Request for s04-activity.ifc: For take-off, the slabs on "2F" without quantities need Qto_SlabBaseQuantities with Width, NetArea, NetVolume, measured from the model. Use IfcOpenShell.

First a look at what the model holds.

```python
import ifcopenshell
import ifcopenshell.util.element
import ifcopenshell.util.unit

model = ifcopenshell.open("s04-activity.ifc")
print(model.schema)
for unit_type in ("LENGTHUNIT", "AREAUNIT", "VOLUMEUNIT"):
    print(unit_type, ifcopenshell.util.unit.calculate_unit_scale(model, unit_type))
storey = next(s for s in model.by_type("IfcBuildingStorey") if s.Name == "2F")
slabs = [e for e in ifcopenshell.util.element.get_decomposition(storey) if e.is_a("IfcSlab")]
for e in sorted(slabs, key=lambda e: e.id()):
    print(e.id(), e.is_a(), e.Name, list(ifcopenshell.util.element.get_psets(e, qtos_only=True)), sep=" | ")
```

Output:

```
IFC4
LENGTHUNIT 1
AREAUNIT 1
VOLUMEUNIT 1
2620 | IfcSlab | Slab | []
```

```python
import ifcopenshell
import ifcopenshell.api.pset
import ifcopenshell.geom
import ifcopenshell.util.element
import ifcopenshell.util.shape
import ifcopenshell.util.unit

model = ifcopenshell.open("s04-activity.ifc")
unit_scale = ifcopenshell.util.unit.calculate_unit_scale(model)
area_scale = ifcopenshell.util.unit.calculate_unit_scale(model, "AREAUNIT")
volume_scale = ifcopenshell.util.unit.calculate_unit_scale(model, "VOLUMEUNIT")
settings = ifcopenshell.geom.settings()

storey = next(s for s in model.by_type("IfcBuildingStorey") if s.Name == "2F")
slabs = [e for e in ifcopenshell.util.element.get_decomposition(storey) if e.is_a("IfcSlab")]

for e in sorted(slabs, key=lambda e: e.id()):
    if ifcopenshell.util.element.get_psets(e, qtos_only=True, should_inherit=False):
        continue
    # Geometry comes back in metres, in the element's own axes.
    shape = ifcopenshell.geom.create_shape(settings, e)
    values = {
        "Width": ifcopenshell.util.shape.get_z(shape.geometry) / unit_scale,
        "NetArea": ifcopenshell.util.shape.get_footprint_area(shape.geometry) / area_scale,
        "NetVolume": ifcopenshell.util.shape.get_volume(shape.geometry) / volume_scale,
    }
    qto = ifcopenshell.api.pset.add_qto(model, product=e, name="Qto_SlabBaseQuantities")
    ifcopenshell.api.pset.edit_qto(model, qto=qto, properties=values)
    print(e.id(), {k: round(v, 3) for k, v in values.items()})

model.write("s04-activity_updated.ifc")
```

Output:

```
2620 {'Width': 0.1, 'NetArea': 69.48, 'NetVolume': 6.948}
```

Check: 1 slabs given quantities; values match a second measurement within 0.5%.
